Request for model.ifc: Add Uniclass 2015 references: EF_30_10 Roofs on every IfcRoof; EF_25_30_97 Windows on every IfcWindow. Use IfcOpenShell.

First a look at what the model holds.

```python
import ifcopenshell

model = ifcopenshell.open("model.ifc")
print(model.schema)
print("classifications:", [c.Name for c in model.by_type("IfcClassification")])
for ifc_class in ("IfcDoor", "IfcRoof", "IfcStair", "IfcWall", "IfcWindow"):
    print(ifc_class, len(model.by_type(ifc_class)))
```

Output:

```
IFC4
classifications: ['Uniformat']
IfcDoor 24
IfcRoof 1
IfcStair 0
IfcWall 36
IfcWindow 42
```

```python
import ifcopenshell
import ifcopenshell.api.classification

model = ifcopenshell.open("model.ifc")

system = ifcopenshell.api.classification.add_classification(model, classification="Uniclass 2015")

codes = {
    "IfcRoof": ("EF_30_10", "Roofs"),
    "IfcWindow": ("EF_25_30_97", "Windows"),
}
for ifc_class, (code, name) in codes.items():
    products = model.by_type(ifc_class)
    ifcopenshell.api.classification.add_reference(
        model, products=products, classification=system, identification=code, name=name
    )
    print(code, len(products))

model.write("model-out.ifc")
```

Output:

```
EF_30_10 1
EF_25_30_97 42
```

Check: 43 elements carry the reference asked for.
